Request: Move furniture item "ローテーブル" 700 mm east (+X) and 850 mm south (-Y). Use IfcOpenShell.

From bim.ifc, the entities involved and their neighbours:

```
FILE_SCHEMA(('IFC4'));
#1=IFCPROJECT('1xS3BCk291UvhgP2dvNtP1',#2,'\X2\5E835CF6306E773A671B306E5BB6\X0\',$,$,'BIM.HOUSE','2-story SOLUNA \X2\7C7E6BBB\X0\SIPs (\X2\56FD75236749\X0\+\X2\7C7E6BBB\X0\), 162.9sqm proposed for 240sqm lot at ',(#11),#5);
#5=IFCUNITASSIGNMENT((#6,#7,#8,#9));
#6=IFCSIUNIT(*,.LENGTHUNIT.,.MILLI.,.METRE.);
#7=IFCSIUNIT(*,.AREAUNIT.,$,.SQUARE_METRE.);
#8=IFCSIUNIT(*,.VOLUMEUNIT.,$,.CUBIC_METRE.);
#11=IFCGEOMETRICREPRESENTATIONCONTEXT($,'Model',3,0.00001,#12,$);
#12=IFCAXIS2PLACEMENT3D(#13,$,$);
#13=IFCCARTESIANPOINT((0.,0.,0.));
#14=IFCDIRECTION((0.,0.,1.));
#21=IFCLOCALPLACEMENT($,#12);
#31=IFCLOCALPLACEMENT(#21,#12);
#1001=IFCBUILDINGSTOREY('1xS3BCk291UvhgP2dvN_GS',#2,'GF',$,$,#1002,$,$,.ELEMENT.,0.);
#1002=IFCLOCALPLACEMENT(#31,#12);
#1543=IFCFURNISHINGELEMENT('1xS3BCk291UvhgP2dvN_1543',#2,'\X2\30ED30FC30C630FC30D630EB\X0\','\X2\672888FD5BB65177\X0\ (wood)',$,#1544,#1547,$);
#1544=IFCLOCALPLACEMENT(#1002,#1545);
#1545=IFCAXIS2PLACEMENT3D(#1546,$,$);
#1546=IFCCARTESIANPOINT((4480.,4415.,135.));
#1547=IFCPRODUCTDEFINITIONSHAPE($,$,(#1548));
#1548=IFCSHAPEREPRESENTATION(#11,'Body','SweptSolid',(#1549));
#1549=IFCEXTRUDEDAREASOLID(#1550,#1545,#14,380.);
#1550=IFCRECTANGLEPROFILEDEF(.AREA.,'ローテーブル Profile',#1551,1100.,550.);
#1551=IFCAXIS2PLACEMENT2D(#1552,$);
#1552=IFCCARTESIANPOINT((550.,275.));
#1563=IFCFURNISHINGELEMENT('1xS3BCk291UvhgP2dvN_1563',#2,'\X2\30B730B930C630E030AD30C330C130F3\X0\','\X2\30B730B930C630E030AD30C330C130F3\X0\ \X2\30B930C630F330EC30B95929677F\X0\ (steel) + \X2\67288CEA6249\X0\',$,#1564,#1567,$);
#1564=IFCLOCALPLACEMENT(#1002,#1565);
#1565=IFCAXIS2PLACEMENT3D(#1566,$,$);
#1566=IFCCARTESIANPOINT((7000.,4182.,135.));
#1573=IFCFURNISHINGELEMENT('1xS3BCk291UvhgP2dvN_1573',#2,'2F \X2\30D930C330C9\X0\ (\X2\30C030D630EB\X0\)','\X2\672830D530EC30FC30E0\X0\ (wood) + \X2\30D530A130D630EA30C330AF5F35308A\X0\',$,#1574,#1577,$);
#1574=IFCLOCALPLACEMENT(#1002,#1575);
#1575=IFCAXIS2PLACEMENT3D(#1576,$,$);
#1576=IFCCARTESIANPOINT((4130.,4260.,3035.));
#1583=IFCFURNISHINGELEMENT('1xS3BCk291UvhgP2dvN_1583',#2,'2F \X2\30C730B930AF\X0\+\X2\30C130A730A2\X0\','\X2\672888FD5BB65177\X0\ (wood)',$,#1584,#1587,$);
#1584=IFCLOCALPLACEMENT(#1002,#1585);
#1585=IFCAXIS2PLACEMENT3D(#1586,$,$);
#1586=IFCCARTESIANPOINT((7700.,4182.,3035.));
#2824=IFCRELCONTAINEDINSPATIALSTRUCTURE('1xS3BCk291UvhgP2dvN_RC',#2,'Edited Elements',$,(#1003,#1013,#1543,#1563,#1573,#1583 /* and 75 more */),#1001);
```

```python
import ifcopenshell
import ifcopenshell.api.geometry
import ifcopenshell.util.placement
import ifcopenshell.util.unit

model = ifcopenshell.open("bim.ifc")
unit_scale = ifcopenshell.util.unit.calculate_unit_scale(model)

item = model.by_guid("1xS3BCk291UvhgP2dvN_1543")
matrix = ifcopenshell.util.placement.get_local_placement(item.ObjectPlacement)
matrix[0, 3] += 0.7 / unit_scale
matrix[1, 3] -= 0.85 / unit_scale
ifcopenshell.api.geometry.edit_object_placement(model, product=item, matrix=matrix, is_si=False)

print(ifcopenshell.util.placement.get_local_placement(item.ObjectPlacement).round(3) + 0.0)

model.write("bim_updated.ifc")
```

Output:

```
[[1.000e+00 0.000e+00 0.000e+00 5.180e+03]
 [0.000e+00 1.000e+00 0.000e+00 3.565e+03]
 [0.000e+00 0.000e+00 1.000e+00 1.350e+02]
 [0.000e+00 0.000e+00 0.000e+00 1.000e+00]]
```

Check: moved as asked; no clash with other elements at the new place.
